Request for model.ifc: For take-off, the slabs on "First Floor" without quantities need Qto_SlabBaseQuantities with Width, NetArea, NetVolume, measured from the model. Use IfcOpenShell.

First a look at what the model holds.

```python
import ifcopenshell
import ifcopenshell.util.element
import ifcopenshell.util.unit

model = ifcopenshell.open("model.ifc")
print(model.schema)
for unit_type in ("LENGTHUNIT", "AREAUNIT", "VOLUMEUNIT"):
    print(unit_type, ifcopenshell.util.unit.calculate_unit_scale(model, unit_type))
storey = next(s for s in model.by_type("IfcBuildingStorey") if s.Name == "First Floor")
slabs = [e for e in ifcopenshell.util.element.get_decomposition(storey) if e.is_a("IfcSlab")]
for e in sorted(slabs, key=lambda e: e.id()):
    print(e.id(), e.is_a(), e.Name, list(ifcopenshell.util.element.get_psets(e, qtos_only=True)), sep=" | ")
```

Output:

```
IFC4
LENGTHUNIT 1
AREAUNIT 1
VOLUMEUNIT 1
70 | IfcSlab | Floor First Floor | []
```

```python
import ifcopenshell
import ifcopenshell.api.pset
import ifcopenshell.geom
import ifcopenshell.util.element
import ifcopenshell.util.shape
import ifcopenshell.util.unit

model = ifcopenshell.open("model.ifc")
unit_scale = ifcopenshell.util.unit.calculate_unit_scale(model)
area_scale = ifcopenshell.util.unit.calculate_unit_scale(model, "AREAUNIT")
volume_scale = ifcopenshell.util.unit.calculate_unit_scale(model, "VOLUMEUNIT")
settings = ifcopenshell.geom.settings()

storey = next(s for s in model.by_type("IfcBuildingStorey") if s.Name == "First Floor")
slabs = [e for e in ifcopenshell.util.element.get_decomposition(storey) if e.is_a("IfcSlab")]

for e in sorted(slabs, key=lambda e: e.id()):
    if ifcopenshell.util.element.get_psets(e, qtos_only=True, should_inherit=False):
        continue
    # Geometry comes back in metres, in the element's own axes.
    shape = ifcopenshell.geom.create_shape(settings, e)
    values = {
        "Width": ifcopenshell.util.shape.get_z(shape.geometry) / unit_scale,
        "NetArea": ifcopenshell.util.shape.get_footprint_area(shape.geometry) / area_scale,
        "NetVolume": ifcopenshell.util.shape.get_volume(shape.geometry) / volume_scale,
    }
    qto = ifcopenshell.api.pset.add_qto(model, product=e, name="Qto_SlabBaseQuantities")
    ifcopenshell.api.pset.edit_qto(model, qto=qto, properties=values)
    print(e.id(), {k: round(v, 3) for k, v in values.items()})

model.write("model_edited.ifc")
```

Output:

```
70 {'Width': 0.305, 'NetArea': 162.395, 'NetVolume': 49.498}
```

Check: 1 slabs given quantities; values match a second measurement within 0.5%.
